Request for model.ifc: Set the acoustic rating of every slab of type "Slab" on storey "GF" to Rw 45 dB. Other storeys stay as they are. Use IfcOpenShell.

First a look at what the model holds.

```python
import ifcopenshell
import ifcopenshell.util.element

model = ifcopenshell.open("model.ifc")
print(model.schema)
storey = next(s for s in model.by_type("IfcBuildingStorey") if s.Name == "GF")
slabs = [e for e in ifcopenshell.util.element.get_decomposition(storey) if e.is_a("IfcSlab")]
seen = {}
for e in slabs:
    element_type = ifcopenshell.util.element.get_type(e)
    key = (element_type.Name if element_type != e and element_type else None, ifcopenshell.util.element.get_pset(e, "Pset_SlabCommon", "AcousticRating"))
    seen[key] = seen.get(key, 0) + 1
for (name, value), count in sorted(seen.items(), key=str):
    print(count, "x", name, "|", value)
```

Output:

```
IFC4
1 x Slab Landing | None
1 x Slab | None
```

```python
import ifcopenshell
import ifcopenshell.api.pset
import ifcopenshell.util.element

model = ifcopenshell.open("model.ifc")

storey = next(s for s in model.by_type("IfcBuildingStorey") if s.Name == "GF")
slabs = [e for e in ifcopenshell.util.element.get_decomposition(storey) if e.is_a("IfcSlab")]

count = 0
for e in slabs:
    element_type = ifcopenshell.util.element.get_type(e)
    if element_type in (None, e) or element_type.Name != "Slab":
        continue
    # add_pset returns the element's existing set when there is one.
    pset = ifcopenshell.api.pset.add_pset(model, product=e, name="Pset_SlabCommon")
    ifcopenshell.api.pset.edit_pset(model, pset=pset, properties={"AcousticRating": "Rw 45 dB"})
    count += 1

print(count, "slabs updated")

model.write("model_rev.ifc")
```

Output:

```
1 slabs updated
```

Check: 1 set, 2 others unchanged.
